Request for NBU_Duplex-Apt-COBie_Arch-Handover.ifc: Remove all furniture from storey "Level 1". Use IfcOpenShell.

First a look at what the model holds.

```python
import ifcopenshell
import ifcopenshell.util.element

model = ifcopenshell.open("NBU_Duplex-Apt-COBie_Arch-Handover.ifc")
print(model.schema)
storey = next(s for s in model.by_type("IfcBuildingStorey") if s.Name == "Level 1")
furniture = [e for e in ifcopenshell.util.element.get_decomposition(storey) if e.is_a("IfcFurnishingElement")]
seen = {}
for e in furniture:
    element_type = ifcopenshell.util.element.get_type(e)
    name = element_type.Name if element_type not in (None, e) else None
    seen[name] = seen.get(name, 0) + 1
for name, count in sorted(seen.items(), key=str):
    print(count, "x", name)
```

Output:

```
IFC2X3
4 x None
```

```python
import ifcopenshell
import ifcopenshell.api.root
import ifcopenshell.util.element

model = ifcopenshell.open("NBU_Duplex-Apt-COBie_Arch-Handover.ifc")

storey = next(s for s in model.by_type("IfcBuildingStorey") if s.Name == "Level 1")
furniture = [e for e in ifcopenshell.util.element.get_decomposition(storey) if e.is_a("IfcFurnishingElement")]

for e in furniture:
    ifcopenshell.api.root.remove_product(model, product=e)
print(len(furniture), "removed")

model.write("NBU_Duplex-Apt-COBie_Arch-Handover_v2.ifc")
```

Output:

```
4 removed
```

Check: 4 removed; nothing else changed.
